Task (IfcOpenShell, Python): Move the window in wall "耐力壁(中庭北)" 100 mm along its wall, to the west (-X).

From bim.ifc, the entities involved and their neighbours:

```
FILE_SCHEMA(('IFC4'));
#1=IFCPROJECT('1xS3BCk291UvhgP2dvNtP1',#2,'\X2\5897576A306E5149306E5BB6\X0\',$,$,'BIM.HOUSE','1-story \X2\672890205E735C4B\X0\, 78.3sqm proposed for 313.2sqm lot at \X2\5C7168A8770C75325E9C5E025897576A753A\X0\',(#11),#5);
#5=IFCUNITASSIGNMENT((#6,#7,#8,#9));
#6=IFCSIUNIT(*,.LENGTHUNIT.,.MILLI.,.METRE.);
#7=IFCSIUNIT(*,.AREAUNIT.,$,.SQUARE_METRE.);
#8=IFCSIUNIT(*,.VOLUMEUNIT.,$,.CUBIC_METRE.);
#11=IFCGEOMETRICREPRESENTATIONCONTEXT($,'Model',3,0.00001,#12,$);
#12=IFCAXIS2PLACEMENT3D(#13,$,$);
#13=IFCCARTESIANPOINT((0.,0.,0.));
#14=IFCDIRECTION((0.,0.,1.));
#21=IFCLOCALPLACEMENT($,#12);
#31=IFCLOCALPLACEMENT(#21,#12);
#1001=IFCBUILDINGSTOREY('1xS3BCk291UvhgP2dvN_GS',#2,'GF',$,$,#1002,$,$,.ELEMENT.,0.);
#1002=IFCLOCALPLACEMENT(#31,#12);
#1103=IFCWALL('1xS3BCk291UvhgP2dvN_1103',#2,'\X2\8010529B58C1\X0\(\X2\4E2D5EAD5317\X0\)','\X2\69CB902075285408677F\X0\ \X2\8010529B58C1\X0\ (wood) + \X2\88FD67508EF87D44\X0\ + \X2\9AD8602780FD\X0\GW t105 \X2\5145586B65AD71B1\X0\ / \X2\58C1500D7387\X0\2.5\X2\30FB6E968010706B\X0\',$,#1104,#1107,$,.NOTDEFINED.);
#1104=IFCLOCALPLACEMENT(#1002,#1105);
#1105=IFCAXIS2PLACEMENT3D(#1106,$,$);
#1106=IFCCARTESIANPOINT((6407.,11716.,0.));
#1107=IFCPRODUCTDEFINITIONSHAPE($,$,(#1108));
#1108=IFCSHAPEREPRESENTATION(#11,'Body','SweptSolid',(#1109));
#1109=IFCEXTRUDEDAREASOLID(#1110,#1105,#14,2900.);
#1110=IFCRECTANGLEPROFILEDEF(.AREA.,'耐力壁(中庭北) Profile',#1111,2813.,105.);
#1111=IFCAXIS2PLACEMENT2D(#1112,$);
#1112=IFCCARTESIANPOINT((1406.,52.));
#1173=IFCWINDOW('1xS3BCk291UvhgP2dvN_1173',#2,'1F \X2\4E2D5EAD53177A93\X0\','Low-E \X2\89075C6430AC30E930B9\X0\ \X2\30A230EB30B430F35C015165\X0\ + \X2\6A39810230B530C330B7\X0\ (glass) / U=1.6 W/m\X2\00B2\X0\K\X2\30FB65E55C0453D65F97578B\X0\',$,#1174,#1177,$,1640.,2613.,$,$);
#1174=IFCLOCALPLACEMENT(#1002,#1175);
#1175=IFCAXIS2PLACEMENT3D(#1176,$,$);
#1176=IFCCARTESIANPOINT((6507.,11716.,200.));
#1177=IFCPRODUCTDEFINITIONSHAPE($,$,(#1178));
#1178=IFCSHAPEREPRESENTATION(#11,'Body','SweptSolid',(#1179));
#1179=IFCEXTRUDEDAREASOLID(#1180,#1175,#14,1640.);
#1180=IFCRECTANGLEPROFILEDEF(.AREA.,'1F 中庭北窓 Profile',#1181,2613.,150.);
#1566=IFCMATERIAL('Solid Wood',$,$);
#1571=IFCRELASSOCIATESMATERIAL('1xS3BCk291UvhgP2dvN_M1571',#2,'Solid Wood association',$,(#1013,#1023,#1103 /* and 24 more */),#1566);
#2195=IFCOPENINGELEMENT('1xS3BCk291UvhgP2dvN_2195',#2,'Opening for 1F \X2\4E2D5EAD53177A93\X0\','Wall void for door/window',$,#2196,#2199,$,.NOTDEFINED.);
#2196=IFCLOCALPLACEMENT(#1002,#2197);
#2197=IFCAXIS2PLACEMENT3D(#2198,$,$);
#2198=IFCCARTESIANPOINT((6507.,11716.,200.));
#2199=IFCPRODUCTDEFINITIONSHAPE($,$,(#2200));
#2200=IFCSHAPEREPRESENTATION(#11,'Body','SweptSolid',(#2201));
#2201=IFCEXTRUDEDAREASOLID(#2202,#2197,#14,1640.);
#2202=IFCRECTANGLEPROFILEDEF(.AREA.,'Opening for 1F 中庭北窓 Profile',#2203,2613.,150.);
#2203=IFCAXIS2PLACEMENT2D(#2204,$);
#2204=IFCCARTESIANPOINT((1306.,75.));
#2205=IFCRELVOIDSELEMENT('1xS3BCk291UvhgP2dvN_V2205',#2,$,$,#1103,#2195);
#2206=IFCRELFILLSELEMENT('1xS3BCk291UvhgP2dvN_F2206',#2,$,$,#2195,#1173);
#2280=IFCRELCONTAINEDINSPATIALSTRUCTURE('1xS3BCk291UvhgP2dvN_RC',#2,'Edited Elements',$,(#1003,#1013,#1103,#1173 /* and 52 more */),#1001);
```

```python
import ifcopenshell
import ifcopenshell.api.geometry
import ifcopenshell.util.placement

model = ifcopenshell.open("bim.ifc")

window = model.by_guid("1xS3BCk291UvhgP2dvN_1173")
opening = window.FillsVoids[0].RelatingOpeningElement
wall = opening.VoidsElements[0].RelatingBuildingElement

wall_matrix = ifcopenshell.util.placement.get_local_placement(wall.ObjectPlacement)
shift = wall_matrix[:3, 0] * -100.0
before = ifcopenshell.util.placement.get_local_placement(window.ObjectPlacement)[:3, 3].copy()

# The window is not placed relative to its opening, so move both.
for product in (opening, window):
    matrix = ifcopenshell.util.placement.get_local_placement(product.ObjectPlacement)
    matrix[:3, 3] += shift
    ifcopenshell.api.geometry.edit_object_placement(model, product=product, matrix=matrix, is_si=False)

after = ifcopenshell.util.placement.get_local_placement(window.ObjectPlacement)[:3, 3]
print("window moved by", (after - before).round(3) + 0.0)

model.write("bim_v2.ifc")
```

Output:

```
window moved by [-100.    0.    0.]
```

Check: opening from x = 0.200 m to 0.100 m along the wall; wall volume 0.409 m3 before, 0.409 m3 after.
